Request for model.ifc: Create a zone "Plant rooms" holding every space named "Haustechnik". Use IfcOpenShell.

First a look at what the model holds.

```python
import ifcopenshell

model = ifcopenshell.open("model.ifc")
print(model.schema)
seen = {}
for space in model.by_type("IfcSpace"):
    seen[space.LongName] = seen.get(space.LongName, 0) + 1
for name, count in sorted(seen.items(), key=str):
    print(count, "x", name)
print("zones:", [z.Name for z in model.by_type("IfcZone")][:20])
```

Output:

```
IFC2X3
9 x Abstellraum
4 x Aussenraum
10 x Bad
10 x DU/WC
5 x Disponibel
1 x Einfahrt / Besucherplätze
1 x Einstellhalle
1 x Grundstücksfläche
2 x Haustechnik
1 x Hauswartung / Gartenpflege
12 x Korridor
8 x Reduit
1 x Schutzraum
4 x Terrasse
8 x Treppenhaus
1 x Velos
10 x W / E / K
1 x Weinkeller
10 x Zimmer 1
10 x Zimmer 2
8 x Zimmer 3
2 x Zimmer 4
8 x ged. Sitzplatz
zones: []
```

```python
import ifcopenshell
import ifcopenshell.api.group
import ifcopenshell.api.root

model = ifcopenshell.open("model.ifc")

names = {"Haustechnik"}
spaces = [s for s in model.by_type("IfcSpace") if s.LongName in names]

zone = ifcopenshell.api.root.create_entity(model, ifc_class="IfcZone", name="Plant rooms")
ifcopenshell.api.group.assign_group(model, products=spaces, group=zone)
print(len(spaces), "spaces in", zone.Name)

model.write("model_rev.ifc")
```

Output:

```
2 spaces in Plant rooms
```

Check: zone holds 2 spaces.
